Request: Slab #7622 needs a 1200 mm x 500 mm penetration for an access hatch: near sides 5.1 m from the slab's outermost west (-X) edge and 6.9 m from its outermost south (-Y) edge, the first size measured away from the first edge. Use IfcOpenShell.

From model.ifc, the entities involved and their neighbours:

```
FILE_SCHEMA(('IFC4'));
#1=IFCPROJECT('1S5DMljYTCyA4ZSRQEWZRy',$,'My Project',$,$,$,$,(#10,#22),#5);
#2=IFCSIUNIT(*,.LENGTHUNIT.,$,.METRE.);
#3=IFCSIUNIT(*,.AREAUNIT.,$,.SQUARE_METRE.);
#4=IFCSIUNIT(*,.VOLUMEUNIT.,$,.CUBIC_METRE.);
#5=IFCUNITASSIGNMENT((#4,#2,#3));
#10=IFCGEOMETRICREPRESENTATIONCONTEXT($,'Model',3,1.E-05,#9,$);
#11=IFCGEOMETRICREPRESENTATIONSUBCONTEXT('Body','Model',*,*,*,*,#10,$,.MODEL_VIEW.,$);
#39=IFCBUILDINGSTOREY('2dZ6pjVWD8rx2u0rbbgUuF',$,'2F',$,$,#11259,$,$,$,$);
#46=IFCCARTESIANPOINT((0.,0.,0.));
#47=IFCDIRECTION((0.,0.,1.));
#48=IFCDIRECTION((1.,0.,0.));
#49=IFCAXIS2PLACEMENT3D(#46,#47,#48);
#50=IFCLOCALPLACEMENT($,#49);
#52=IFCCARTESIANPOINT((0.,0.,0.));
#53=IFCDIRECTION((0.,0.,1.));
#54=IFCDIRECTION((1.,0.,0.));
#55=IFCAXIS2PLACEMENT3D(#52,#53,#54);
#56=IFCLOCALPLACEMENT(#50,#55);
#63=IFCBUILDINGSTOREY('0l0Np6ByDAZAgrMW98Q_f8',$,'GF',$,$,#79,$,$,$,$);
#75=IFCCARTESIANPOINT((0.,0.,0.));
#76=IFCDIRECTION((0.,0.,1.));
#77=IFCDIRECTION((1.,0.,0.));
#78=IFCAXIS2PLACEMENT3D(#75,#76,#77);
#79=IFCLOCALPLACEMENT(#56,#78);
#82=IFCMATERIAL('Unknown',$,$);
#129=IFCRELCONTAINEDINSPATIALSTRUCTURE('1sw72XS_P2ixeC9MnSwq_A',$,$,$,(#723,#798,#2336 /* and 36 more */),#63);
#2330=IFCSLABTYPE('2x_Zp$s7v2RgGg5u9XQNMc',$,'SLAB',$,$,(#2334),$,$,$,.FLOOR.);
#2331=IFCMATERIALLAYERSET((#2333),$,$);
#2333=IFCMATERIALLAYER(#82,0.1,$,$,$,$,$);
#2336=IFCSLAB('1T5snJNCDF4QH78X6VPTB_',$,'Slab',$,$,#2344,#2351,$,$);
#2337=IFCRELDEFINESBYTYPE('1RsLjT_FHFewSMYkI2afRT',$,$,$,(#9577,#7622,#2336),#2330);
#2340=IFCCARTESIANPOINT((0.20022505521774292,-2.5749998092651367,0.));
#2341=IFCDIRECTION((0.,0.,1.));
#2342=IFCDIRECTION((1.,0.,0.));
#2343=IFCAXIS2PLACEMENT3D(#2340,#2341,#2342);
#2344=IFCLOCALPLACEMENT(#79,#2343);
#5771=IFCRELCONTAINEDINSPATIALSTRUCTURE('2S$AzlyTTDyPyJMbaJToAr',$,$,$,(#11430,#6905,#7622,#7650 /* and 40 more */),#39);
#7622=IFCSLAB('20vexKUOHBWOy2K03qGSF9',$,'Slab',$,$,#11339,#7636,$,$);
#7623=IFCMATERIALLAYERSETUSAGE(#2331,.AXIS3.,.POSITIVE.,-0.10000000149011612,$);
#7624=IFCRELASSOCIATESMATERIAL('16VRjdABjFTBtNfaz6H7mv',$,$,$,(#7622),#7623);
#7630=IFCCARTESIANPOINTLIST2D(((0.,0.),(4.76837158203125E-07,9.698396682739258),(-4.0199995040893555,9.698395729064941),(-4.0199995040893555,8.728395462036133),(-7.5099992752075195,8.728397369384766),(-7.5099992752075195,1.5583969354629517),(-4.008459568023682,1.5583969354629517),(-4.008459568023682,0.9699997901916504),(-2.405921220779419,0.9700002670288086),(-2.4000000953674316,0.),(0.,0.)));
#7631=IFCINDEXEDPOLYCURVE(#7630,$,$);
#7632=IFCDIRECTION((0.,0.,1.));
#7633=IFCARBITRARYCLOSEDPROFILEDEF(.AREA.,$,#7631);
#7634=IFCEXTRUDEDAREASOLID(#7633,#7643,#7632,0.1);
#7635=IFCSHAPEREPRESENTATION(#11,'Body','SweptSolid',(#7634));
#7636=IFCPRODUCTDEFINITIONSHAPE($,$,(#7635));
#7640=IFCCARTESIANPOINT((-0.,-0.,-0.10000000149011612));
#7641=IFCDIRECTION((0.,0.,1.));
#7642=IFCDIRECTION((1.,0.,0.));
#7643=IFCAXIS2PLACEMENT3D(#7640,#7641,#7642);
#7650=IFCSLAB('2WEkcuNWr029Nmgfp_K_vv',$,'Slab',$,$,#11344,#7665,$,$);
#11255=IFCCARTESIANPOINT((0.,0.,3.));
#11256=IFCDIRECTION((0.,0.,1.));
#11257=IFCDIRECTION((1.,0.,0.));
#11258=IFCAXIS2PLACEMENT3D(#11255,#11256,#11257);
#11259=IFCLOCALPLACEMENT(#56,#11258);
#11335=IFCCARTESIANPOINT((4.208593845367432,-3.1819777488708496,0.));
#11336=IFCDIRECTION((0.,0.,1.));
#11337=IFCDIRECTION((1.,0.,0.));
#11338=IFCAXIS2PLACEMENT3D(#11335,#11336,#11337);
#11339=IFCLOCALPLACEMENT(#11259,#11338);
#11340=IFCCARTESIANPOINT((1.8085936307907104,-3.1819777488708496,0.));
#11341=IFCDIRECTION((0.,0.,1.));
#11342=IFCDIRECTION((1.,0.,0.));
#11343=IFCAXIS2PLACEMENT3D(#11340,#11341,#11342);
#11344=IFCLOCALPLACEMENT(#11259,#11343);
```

```python
import numpy as np
import ifcopenshell
import ifcopenshell.api.feature
import ifcopenshell.api.geometry
import ifcopenshell.api.root
import ifcopenshell.geom
import ifcopenshell.util.placement
import ifcopenshell.util.representation
import ifcopenshell.util.shape
import ifcopenshell.util.unit

model = ifcopenshell.open("model.ifc")
unit_scale = ifcopenshell.util.unit.calculate_unit_scale(model)
settings = ifcopenshell.geom.settings()


def volume(element):
    """Net volume in cubic metres, openings subtracted."""
    shape = ifcopenshell.geom.create_shape(settings, element)
    return ifcopenshell.util.shape.get_volume(shape.geometry)


slab = model.by_guid("20vexKUOHBWOy2K03qGSF9")
before = volume(slab)

# Extent in the slab's own axes, in metres. The edges named are its -X and -Y sides.
slab_shape = ifcopenshell.geom.create_shape(settings, slab)
vertices = ifcopenshell.util.shape.get_vertices(slab_shape.geometry)
x_min, y_min, bottom = vertices.min(axis=0)
top = vertices[:, 2].max()

opening = ifcopenshell.api.root.create_entity(model, ifc_class="IfcOpeningElement", name="Access hatch opening", predefined_type="OPENING")
context = ifcopenshell.util.representation.get_context(model, "Model", "Body", "MODEL_VIEW")
width, depth = 1.2, 0.5
outline = [(0.0, 0.0), (width, 0.0), (width, depth), (0.0, depth), (0.0, 0.0)]
# Overshoot both faces by 50 mm so the cut is clean.
shape = ifcopenshell.api.geometry.add_slab_representation(
    model, context=context, depth=top - bottom + 0.1, polyline=outline
)
ifcopenshell.api.geometry.assign_representation(model, product=opening, representation=shape)

matrix = ifcopenshell.util.placement.get_local_placement(slab.ObjectPlacement)
matrix[:, 3] = matrix @ np.append(np.array([x_min + 5.1, y_min + 6.9, bottom - 0.05]) / unit_scale, 1.0)
ifcopenshell.api.geometry.edit_object_placement(model, product=opening, matrix=matrix, is_si=False)
ifcopenshell.api.feature.add_feature(model, feature=opening, element=slab)

after = volume(slab)

print(f"slab volume {before:.3f} -> {after:.3f} m3")

model.write("model_edited.ifc")
```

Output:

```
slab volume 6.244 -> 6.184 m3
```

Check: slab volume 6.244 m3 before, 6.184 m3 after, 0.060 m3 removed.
